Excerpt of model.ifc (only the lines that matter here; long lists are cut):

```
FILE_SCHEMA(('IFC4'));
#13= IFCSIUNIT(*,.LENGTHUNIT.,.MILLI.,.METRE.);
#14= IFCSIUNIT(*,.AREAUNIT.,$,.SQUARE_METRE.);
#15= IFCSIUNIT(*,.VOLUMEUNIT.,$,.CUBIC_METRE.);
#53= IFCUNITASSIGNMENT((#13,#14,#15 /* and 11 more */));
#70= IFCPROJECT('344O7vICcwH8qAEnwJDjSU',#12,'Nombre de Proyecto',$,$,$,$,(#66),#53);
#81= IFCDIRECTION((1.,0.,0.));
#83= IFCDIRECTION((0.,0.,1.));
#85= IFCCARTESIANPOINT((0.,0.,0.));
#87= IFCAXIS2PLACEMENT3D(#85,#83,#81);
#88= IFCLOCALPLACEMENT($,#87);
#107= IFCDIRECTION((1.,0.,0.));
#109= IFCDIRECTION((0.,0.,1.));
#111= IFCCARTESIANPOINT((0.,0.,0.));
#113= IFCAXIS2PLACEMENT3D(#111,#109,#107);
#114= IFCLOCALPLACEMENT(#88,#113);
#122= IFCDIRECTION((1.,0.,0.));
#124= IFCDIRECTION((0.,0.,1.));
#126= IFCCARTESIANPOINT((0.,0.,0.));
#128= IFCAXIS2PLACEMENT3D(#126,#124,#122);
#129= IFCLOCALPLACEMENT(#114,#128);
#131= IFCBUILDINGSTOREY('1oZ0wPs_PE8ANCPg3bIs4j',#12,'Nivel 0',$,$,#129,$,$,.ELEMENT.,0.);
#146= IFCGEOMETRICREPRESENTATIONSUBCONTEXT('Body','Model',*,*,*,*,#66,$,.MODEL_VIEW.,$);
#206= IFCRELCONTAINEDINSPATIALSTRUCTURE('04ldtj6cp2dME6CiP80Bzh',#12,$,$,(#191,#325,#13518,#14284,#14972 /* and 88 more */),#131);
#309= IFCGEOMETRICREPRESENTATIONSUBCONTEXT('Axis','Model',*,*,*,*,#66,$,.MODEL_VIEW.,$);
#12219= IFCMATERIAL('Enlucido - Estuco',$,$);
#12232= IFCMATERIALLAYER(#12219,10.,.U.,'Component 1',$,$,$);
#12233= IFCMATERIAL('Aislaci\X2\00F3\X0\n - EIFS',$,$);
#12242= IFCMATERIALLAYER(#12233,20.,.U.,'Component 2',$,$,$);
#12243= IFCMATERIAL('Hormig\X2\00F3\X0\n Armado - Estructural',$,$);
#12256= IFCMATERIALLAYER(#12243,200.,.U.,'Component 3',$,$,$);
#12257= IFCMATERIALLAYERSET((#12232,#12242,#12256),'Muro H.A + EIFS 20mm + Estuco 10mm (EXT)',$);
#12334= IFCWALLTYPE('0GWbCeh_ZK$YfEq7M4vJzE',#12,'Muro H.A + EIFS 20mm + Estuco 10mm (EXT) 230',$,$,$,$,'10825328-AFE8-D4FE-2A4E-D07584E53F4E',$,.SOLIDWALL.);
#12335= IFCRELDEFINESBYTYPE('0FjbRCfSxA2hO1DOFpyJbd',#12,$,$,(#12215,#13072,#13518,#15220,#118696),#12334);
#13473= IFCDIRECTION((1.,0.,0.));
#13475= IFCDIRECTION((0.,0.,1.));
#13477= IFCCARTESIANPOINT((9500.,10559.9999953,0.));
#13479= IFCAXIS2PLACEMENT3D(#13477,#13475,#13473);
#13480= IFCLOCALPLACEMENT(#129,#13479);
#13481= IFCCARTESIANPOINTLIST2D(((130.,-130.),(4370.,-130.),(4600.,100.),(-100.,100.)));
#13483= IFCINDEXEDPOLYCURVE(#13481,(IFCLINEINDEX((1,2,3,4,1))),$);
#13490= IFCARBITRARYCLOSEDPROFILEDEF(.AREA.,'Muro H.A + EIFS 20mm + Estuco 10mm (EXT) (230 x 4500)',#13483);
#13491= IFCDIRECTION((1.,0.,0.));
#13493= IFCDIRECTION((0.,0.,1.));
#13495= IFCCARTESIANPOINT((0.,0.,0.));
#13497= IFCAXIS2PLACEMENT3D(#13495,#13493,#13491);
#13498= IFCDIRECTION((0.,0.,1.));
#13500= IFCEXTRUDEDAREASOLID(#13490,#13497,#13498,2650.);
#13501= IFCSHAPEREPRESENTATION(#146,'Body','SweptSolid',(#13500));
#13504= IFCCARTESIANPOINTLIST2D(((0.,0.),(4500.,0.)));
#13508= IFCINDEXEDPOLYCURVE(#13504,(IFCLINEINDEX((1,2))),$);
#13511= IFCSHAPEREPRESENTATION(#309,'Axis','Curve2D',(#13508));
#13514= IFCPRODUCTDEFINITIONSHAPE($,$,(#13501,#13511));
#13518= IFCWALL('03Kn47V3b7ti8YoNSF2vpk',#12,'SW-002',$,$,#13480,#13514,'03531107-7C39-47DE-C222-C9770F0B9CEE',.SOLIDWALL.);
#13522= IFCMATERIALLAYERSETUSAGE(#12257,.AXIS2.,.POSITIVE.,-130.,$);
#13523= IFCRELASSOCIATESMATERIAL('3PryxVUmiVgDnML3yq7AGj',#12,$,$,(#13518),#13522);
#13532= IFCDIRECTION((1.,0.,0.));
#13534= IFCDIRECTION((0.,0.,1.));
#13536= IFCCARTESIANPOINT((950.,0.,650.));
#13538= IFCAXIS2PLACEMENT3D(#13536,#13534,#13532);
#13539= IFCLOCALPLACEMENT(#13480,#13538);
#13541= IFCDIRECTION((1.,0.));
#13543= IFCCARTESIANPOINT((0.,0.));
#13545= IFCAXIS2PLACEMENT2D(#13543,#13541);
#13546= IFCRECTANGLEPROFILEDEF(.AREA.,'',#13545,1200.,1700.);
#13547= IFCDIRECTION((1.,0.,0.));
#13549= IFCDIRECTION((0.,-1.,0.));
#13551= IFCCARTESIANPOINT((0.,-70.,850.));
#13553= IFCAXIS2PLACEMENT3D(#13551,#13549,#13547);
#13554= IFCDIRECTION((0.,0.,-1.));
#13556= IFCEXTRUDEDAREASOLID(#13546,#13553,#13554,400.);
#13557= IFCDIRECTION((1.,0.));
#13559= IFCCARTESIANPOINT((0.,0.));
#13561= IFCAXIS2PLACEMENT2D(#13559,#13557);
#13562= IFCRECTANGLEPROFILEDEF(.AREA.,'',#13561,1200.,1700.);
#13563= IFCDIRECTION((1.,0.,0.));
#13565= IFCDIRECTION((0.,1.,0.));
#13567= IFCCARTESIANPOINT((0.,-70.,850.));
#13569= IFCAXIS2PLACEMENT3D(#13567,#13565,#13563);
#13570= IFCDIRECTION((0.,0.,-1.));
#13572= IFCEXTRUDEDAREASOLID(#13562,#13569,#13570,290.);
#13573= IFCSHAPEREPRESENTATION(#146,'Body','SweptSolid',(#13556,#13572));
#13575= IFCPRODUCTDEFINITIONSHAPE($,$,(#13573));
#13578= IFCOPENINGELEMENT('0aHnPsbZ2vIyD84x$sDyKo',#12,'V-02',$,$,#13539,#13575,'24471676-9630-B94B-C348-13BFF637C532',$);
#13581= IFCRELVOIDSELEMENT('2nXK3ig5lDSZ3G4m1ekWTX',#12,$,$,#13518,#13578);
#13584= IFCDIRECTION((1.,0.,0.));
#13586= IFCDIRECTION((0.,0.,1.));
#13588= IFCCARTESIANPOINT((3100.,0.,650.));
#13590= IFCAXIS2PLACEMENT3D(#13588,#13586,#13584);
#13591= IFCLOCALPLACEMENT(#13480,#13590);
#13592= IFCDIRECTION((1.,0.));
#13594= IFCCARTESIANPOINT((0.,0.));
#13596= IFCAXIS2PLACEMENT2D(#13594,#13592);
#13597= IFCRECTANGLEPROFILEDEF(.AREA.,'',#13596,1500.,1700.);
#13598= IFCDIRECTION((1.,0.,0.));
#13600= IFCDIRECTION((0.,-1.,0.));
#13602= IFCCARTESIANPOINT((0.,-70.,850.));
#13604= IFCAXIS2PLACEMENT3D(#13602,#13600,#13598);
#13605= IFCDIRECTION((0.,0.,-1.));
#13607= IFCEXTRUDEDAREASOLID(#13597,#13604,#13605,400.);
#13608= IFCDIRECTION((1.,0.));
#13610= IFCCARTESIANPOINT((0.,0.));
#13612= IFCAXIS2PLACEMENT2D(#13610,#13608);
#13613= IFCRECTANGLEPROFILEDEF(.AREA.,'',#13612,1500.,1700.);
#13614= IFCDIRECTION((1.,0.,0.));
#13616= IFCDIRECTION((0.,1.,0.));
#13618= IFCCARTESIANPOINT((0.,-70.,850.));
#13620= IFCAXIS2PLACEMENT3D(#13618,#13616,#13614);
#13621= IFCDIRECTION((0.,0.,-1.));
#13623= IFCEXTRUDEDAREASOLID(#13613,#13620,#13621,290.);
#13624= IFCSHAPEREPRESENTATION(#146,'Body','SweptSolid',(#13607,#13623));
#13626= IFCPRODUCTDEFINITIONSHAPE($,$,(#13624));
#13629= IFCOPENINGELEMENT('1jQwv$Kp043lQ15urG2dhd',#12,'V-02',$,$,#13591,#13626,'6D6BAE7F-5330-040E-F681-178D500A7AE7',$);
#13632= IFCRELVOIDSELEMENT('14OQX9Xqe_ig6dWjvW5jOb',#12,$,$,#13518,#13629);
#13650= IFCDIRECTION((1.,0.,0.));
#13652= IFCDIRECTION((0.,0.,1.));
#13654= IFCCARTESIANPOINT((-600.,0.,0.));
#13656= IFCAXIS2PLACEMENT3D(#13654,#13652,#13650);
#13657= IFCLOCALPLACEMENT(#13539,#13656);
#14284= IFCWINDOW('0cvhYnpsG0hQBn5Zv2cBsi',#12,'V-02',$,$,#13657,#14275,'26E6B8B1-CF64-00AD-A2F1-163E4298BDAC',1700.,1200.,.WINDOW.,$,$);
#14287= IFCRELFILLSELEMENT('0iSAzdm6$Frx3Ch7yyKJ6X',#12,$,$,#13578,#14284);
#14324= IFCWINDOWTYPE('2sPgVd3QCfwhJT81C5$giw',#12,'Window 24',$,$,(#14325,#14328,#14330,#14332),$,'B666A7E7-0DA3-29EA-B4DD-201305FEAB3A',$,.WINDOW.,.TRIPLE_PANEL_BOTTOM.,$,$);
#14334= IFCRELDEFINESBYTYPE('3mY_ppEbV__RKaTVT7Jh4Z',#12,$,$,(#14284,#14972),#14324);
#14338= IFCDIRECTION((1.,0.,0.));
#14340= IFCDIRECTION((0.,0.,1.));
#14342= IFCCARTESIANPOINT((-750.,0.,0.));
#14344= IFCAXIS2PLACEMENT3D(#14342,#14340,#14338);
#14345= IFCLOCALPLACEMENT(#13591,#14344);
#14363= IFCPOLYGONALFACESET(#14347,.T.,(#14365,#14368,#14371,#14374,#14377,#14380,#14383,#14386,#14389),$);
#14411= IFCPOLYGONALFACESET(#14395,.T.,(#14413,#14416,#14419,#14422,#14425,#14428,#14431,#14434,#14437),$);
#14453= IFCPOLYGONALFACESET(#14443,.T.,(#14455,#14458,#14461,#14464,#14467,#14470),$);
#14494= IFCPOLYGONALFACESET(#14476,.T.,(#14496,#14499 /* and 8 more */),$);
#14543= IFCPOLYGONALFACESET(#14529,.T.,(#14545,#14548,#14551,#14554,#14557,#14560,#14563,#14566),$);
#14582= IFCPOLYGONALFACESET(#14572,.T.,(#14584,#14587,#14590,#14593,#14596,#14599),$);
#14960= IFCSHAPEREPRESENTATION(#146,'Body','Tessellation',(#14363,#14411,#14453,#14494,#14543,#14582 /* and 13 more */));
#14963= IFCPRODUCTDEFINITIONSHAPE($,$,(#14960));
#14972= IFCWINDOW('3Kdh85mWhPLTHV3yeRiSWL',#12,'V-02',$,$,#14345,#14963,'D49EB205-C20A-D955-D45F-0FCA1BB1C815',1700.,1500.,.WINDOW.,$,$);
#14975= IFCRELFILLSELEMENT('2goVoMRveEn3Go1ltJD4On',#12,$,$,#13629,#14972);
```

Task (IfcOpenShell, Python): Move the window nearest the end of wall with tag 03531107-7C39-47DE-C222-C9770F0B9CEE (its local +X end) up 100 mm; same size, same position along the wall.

```python
import numpy as np
import ifcopenshell
import ifcopenshell.api.geometry
import ifcopenshell.util.placement
import ifcopenshell.util.unit

model = ifcopenshell.open("model.ifc")
unit_scale = ifcopenshell.util.unit.calculate_unit_scale(model)

window = model.by_guid("3Kdh85mWhPLTHV3yeRiSWL")
opening = window.FillsVoids[0].RelatingOpeningElement
dz = 0.1 / unit_scale

shift = np.array([0.0, 0.0, dz])
# The window is placed relative to its opening, so it follows when the opening moves.
matrix = ifcopenshell.util.placement.get_local_placement(opening.ObjectPlacement)
matrix[:3, 3] += shift
ifcopenshell.api.geometry.edit_object_placement(
    model, product=opening, matrix=matrix, is_si=False, should_transform_children=True
)

print(f"moved by {dz * unit_scale:+.3f} m")

model.write("model_edited.ifc")
```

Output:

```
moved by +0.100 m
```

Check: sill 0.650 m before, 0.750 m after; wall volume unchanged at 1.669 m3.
